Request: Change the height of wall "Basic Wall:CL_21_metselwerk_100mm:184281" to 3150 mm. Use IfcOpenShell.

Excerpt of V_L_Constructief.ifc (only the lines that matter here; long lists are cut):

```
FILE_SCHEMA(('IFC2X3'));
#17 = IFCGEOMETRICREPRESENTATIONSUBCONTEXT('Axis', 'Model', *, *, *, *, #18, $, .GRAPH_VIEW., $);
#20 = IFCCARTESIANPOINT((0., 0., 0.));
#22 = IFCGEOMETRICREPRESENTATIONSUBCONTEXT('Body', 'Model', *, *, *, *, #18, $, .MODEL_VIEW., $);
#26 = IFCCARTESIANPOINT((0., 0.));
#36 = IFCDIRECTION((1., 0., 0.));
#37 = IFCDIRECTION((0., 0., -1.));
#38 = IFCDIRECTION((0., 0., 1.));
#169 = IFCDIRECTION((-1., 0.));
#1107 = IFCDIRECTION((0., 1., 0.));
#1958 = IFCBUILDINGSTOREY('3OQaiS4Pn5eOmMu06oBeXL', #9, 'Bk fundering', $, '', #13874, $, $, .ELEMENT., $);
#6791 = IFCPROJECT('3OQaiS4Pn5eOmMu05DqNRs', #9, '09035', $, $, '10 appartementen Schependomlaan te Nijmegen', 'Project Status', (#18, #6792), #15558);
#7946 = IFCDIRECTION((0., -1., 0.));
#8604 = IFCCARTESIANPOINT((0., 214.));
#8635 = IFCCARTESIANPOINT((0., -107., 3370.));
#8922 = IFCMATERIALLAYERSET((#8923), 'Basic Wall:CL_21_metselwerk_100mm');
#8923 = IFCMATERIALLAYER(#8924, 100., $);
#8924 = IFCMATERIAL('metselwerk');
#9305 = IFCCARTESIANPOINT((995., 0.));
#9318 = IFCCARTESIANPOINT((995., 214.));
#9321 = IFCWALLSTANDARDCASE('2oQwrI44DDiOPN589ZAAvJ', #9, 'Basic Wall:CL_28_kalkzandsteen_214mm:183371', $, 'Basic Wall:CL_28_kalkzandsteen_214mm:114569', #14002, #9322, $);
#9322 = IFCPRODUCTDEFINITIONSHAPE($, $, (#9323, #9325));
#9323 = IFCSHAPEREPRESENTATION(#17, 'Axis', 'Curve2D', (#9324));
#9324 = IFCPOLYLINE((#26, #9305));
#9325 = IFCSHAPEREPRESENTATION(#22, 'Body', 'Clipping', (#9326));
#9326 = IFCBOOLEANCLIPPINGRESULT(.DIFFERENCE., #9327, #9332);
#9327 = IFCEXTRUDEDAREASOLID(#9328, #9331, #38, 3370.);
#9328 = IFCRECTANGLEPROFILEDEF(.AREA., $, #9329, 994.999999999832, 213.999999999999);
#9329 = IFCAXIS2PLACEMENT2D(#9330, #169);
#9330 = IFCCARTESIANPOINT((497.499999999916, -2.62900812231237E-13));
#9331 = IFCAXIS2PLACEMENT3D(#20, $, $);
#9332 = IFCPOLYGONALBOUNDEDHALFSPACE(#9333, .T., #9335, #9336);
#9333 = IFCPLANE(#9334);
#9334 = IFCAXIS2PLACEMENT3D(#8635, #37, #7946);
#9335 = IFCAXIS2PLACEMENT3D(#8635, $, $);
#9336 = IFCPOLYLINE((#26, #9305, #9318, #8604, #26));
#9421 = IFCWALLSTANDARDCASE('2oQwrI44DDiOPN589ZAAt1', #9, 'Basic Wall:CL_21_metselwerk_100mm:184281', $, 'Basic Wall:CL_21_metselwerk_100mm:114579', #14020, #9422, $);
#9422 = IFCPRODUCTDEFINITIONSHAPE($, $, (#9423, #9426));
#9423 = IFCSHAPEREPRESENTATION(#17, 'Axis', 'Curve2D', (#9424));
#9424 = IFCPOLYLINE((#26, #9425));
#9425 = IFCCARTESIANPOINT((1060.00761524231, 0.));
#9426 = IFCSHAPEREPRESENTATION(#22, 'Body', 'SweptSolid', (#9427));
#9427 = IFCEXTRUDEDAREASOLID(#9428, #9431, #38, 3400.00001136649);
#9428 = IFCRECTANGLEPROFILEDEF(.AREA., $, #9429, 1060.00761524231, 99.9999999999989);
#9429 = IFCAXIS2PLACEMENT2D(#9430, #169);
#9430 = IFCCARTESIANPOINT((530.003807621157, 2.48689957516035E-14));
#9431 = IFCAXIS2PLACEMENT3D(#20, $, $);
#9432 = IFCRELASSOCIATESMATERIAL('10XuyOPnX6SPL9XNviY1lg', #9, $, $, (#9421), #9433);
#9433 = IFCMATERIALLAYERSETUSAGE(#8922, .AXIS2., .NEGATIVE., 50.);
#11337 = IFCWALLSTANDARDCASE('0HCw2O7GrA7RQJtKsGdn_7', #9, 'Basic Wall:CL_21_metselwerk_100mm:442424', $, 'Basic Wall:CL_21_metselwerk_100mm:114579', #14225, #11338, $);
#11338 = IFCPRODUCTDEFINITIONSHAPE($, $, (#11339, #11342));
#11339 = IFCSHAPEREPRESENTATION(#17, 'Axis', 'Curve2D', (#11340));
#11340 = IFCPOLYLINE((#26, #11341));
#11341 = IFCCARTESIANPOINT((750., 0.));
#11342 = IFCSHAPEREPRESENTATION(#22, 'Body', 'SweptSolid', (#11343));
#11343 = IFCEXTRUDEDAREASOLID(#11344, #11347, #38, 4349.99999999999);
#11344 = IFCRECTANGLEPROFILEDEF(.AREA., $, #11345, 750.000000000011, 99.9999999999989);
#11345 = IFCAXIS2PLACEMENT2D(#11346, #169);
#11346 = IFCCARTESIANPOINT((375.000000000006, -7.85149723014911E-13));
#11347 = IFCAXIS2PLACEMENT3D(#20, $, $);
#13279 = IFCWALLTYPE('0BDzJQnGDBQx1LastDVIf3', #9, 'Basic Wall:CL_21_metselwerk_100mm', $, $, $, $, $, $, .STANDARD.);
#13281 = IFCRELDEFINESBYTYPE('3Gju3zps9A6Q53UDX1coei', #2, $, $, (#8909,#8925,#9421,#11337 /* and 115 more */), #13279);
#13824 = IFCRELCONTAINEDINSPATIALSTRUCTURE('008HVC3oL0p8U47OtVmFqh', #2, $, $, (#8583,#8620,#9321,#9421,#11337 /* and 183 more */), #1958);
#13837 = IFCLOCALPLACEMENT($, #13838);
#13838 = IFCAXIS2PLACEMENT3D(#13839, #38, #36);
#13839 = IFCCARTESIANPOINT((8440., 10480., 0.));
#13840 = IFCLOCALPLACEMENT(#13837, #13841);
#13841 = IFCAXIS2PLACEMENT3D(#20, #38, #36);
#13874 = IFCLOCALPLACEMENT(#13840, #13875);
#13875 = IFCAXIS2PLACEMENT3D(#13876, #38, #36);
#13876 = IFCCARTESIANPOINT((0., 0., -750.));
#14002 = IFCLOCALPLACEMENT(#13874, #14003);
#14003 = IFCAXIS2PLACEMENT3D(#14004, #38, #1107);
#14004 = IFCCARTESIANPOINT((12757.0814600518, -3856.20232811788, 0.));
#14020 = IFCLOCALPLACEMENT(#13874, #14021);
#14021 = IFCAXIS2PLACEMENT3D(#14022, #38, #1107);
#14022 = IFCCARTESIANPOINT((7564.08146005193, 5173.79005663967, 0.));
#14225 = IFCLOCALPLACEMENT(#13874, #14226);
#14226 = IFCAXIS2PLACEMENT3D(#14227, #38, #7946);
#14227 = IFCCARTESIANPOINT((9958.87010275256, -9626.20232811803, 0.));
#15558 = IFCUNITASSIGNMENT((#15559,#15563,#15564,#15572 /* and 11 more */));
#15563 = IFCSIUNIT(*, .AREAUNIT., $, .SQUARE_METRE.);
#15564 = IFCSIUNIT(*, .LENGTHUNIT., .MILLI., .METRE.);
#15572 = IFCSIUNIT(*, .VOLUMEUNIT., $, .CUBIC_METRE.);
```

```python
import ifcopenshell
import ifcopenshell.geom
import ifcopenshell.util.representation
import ifcopenshell.util.shape

model = ifcopenshell.open("V_L_Constructief.ifc")
settings = ifcopenshell.geom.settings()


def volume(element):
    """Net volume in cubic metres, openings subtracted."""
    shape = ifcopenshell.geom.create_shape(settings, element)
    return ifcopenshell.util.shape.get_volume(shape.geometry)


wall = model.by_guid("2oQwrI44DDiOPN589ZAAt1")
before = volume(wall)

body = ifcopenshell.util.representation.get_representation(wall, "Model", "Body")
solid = body.Items[0]
old_height = solid.Depth
solid.Depth = 3150.0
after = volume(wall)

print(f"height {old_height:g} -> {solid.Depth:g}, volume {before:.3f} -> {after:.3f} m3")

model.write("V_L_Constructief_rev.ifc")
```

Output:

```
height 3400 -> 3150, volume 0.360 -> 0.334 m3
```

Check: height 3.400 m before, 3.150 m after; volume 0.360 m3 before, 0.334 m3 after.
